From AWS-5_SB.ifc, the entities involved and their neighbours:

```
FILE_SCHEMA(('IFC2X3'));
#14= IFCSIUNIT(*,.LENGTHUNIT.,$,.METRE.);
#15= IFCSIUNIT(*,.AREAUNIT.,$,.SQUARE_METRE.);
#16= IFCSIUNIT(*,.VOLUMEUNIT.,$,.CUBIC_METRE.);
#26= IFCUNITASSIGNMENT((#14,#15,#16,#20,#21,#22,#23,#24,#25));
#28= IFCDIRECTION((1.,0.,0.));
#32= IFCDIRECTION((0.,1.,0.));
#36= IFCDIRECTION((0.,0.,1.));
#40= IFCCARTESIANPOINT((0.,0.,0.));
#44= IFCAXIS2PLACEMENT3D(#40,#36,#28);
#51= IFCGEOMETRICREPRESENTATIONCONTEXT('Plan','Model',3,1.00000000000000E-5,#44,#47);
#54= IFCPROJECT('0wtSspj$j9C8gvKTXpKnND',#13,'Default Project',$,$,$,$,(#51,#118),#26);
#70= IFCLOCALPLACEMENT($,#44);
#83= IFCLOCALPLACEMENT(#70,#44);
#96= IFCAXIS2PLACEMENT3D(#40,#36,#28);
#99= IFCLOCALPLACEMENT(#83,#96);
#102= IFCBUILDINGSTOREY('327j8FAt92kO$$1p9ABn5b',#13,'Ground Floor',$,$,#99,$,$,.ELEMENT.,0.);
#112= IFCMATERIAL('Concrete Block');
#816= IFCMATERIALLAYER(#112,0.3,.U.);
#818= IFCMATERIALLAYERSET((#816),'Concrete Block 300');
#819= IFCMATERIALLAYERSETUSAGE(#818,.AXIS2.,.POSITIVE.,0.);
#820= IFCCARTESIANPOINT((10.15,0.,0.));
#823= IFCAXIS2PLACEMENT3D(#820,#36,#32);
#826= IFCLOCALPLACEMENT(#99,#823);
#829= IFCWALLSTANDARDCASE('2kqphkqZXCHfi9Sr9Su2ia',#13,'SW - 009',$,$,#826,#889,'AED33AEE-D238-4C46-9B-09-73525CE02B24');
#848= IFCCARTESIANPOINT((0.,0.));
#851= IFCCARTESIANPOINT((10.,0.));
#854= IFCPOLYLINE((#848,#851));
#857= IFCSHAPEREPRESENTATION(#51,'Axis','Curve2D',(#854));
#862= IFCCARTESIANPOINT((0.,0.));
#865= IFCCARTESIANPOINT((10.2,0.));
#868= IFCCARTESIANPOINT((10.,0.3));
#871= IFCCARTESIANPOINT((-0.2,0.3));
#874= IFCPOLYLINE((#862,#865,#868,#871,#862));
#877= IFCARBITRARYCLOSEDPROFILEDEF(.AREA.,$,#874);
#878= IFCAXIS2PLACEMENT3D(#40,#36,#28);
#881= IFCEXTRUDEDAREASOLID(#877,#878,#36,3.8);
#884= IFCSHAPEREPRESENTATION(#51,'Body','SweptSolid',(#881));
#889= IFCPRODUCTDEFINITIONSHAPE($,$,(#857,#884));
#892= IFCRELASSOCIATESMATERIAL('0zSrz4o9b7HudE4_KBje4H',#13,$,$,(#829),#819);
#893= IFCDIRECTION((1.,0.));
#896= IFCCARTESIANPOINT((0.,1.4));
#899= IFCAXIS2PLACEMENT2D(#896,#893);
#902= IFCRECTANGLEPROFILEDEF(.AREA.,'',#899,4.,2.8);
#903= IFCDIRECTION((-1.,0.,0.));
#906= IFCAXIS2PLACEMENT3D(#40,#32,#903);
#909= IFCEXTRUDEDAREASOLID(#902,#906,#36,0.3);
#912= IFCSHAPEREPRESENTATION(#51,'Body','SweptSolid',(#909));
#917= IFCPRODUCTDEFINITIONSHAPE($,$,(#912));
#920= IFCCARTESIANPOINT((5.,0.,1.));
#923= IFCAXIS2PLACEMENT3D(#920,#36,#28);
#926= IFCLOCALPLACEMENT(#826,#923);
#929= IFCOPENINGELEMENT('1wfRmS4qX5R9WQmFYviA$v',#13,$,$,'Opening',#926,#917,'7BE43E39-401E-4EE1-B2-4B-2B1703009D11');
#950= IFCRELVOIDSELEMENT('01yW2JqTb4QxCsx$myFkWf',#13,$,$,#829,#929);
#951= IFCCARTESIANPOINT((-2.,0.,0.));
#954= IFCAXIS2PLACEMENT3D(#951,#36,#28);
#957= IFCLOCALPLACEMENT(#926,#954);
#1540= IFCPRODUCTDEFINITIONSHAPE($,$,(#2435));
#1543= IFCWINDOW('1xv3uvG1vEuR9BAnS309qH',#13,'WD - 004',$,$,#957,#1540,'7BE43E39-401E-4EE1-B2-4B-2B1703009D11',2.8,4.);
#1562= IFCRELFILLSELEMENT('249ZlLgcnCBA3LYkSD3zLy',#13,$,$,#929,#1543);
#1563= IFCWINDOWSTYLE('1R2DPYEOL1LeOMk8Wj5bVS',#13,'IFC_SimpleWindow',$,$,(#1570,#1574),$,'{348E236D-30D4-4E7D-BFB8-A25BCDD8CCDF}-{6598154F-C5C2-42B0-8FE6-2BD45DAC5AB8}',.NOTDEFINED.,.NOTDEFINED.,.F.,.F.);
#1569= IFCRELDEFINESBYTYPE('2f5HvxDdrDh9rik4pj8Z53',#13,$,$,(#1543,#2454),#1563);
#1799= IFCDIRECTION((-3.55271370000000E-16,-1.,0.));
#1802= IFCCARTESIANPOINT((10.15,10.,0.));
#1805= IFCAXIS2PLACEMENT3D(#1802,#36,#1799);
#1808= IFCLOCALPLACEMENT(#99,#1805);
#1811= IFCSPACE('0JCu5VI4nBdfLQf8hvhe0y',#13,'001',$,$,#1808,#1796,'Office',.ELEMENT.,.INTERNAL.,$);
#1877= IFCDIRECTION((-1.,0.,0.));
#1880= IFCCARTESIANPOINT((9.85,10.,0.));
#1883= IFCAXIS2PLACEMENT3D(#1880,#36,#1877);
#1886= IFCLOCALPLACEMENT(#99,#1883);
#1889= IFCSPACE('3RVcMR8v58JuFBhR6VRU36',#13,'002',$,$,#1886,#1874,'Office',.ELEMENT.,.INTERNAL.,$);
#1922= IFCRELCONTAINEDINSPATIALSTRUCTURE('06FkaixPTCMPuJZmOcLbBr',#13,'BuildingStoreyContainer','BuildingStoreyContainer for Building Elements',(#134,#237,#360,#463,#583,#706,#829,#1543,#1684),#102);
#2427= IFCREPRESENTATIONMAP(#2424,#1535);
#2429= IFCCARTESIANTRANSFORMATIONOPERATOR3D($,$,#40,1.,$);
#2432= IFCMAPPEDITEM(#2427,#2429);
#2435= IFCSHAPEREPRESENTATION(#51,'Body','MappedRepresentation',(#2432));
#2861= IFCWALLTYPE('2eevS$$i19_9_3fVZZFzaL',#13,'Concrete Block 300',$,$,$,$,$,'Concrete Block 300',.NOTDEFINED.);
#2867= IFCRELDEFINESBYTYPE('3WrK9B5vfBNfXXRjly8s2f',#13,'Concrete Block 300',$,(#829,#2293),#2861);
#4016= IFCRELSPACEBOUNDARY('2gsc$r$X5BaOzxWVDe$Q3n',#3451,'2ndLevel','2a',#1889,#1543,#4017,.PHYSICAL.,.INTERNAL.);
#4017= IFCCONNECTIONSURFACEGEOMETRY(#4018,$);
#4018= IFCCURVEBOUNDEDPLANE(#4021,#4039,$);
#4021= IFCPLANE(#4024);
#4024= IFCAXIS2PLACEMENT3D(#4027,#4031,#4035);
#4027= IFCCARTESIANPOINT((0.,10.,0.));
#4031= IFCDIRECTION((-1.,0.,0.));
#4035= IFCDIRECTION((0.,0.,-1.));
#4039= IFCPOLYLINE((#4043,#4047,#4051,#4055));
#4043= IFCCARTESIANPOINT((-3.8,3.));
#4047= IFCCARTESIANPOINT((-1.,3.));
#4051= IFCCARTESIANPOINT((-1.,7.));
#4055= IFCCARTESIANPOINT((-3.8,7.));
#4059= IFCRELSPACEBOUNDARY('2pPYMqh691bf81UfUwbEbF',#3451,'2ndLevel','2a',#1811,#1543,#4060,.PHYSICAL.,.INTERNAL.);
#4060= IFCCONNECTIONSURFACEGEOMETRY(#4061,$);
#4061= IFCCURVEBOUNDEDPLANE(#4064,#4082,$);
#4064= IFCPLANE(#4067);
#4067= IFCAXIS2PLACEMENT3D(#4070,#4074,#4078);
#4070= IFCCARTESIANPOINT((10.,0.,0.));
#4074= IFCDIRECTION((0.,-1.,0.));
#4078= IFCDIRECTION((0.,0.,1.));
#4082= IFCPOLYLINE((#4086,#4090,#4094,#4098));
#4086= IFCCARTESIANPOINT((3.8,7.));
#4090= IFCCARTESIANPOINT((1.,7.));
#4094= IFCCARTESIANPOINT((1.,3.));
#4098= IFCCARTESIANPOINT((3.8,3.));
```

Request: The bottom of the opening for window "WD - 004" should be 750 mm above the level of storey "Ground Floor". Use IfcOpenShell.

```python
import numpy as np
import ifcopenshell
import ifcopenshell.api.geometry
import ifcopenshell.geom
import ifcopenshell.util.element
import ifcopenshell.util.placement
import ifcopenshell.util.shape
import ifcopenshell.util.unit

model = ifcopenshell.open("AWS-5_SB.ifc")
unit_scale = ifcopenshell.util.unit.calculate_unit_scale(model)

window = model.by_id(1543)
opening = window.FillsVoids[0].RelatingOpeningElement
storey = ifcopenshell.util.element.get_container(window, ifc_class="IfcBuildingStorey")
level = ifcopenshell.util.placement.get_local_placement(storey.ObjectPlacement)[2, 3]

# The opening's origin need not be at the sill, so measure its lowest point.
shape = ifcopenshell.geom.create_shape(ifcopenshell.geom.settings(), opening)
bottom = ifcopenshell.util.shape.get_shape_bottom_elevation(shape, shape.geometry) / unit_scale
dz = level + 0.75 - bottom

shift = np.array([0.0, 0.0, dz])
# The window is placed relative to its opening, so it follows when the opening moves.
matrix = ifcopenshell.util.placement.get_local_placement(opening.ObjectPlacement)
matrix[:3, 3] += shift
ifcopenshell.api.geometry.edit_object_placement(
    model, product=opening, matrix=matrix, is_si=False, should_transform_children=True
)

# Space boundary surfaces are stored in each space's coordinates; move them too.
for rel in window.ProvidesBoundaries:
    if not rel.ConnectionGeometry:
        continue
    surface = rel.ConnectionGeometry.SurfaceOnRelatingElement.BasisSurface
    space_matrix = ifcopenshell.util.placement.get_local_placement(rel.RelatingSpace.ObjectPlacement)
    point = np.array(surface.Position.Location.Coordinates) + space_matrix[:3, :3].T @ shift
    surface.Position = model.createIfcAxis2Placement3D(
        model.createIfcCartesianPoint(point.tolist()), surface.Position.Axis, surface.Position.RefDirection
    )

print(f"moved by {dz * unit_scale:+.3f} m")

model.write("AWS-5_SB-out.ifc")
```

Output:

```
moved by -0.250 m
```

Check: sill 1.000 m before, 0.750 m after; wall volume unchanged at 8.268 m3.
